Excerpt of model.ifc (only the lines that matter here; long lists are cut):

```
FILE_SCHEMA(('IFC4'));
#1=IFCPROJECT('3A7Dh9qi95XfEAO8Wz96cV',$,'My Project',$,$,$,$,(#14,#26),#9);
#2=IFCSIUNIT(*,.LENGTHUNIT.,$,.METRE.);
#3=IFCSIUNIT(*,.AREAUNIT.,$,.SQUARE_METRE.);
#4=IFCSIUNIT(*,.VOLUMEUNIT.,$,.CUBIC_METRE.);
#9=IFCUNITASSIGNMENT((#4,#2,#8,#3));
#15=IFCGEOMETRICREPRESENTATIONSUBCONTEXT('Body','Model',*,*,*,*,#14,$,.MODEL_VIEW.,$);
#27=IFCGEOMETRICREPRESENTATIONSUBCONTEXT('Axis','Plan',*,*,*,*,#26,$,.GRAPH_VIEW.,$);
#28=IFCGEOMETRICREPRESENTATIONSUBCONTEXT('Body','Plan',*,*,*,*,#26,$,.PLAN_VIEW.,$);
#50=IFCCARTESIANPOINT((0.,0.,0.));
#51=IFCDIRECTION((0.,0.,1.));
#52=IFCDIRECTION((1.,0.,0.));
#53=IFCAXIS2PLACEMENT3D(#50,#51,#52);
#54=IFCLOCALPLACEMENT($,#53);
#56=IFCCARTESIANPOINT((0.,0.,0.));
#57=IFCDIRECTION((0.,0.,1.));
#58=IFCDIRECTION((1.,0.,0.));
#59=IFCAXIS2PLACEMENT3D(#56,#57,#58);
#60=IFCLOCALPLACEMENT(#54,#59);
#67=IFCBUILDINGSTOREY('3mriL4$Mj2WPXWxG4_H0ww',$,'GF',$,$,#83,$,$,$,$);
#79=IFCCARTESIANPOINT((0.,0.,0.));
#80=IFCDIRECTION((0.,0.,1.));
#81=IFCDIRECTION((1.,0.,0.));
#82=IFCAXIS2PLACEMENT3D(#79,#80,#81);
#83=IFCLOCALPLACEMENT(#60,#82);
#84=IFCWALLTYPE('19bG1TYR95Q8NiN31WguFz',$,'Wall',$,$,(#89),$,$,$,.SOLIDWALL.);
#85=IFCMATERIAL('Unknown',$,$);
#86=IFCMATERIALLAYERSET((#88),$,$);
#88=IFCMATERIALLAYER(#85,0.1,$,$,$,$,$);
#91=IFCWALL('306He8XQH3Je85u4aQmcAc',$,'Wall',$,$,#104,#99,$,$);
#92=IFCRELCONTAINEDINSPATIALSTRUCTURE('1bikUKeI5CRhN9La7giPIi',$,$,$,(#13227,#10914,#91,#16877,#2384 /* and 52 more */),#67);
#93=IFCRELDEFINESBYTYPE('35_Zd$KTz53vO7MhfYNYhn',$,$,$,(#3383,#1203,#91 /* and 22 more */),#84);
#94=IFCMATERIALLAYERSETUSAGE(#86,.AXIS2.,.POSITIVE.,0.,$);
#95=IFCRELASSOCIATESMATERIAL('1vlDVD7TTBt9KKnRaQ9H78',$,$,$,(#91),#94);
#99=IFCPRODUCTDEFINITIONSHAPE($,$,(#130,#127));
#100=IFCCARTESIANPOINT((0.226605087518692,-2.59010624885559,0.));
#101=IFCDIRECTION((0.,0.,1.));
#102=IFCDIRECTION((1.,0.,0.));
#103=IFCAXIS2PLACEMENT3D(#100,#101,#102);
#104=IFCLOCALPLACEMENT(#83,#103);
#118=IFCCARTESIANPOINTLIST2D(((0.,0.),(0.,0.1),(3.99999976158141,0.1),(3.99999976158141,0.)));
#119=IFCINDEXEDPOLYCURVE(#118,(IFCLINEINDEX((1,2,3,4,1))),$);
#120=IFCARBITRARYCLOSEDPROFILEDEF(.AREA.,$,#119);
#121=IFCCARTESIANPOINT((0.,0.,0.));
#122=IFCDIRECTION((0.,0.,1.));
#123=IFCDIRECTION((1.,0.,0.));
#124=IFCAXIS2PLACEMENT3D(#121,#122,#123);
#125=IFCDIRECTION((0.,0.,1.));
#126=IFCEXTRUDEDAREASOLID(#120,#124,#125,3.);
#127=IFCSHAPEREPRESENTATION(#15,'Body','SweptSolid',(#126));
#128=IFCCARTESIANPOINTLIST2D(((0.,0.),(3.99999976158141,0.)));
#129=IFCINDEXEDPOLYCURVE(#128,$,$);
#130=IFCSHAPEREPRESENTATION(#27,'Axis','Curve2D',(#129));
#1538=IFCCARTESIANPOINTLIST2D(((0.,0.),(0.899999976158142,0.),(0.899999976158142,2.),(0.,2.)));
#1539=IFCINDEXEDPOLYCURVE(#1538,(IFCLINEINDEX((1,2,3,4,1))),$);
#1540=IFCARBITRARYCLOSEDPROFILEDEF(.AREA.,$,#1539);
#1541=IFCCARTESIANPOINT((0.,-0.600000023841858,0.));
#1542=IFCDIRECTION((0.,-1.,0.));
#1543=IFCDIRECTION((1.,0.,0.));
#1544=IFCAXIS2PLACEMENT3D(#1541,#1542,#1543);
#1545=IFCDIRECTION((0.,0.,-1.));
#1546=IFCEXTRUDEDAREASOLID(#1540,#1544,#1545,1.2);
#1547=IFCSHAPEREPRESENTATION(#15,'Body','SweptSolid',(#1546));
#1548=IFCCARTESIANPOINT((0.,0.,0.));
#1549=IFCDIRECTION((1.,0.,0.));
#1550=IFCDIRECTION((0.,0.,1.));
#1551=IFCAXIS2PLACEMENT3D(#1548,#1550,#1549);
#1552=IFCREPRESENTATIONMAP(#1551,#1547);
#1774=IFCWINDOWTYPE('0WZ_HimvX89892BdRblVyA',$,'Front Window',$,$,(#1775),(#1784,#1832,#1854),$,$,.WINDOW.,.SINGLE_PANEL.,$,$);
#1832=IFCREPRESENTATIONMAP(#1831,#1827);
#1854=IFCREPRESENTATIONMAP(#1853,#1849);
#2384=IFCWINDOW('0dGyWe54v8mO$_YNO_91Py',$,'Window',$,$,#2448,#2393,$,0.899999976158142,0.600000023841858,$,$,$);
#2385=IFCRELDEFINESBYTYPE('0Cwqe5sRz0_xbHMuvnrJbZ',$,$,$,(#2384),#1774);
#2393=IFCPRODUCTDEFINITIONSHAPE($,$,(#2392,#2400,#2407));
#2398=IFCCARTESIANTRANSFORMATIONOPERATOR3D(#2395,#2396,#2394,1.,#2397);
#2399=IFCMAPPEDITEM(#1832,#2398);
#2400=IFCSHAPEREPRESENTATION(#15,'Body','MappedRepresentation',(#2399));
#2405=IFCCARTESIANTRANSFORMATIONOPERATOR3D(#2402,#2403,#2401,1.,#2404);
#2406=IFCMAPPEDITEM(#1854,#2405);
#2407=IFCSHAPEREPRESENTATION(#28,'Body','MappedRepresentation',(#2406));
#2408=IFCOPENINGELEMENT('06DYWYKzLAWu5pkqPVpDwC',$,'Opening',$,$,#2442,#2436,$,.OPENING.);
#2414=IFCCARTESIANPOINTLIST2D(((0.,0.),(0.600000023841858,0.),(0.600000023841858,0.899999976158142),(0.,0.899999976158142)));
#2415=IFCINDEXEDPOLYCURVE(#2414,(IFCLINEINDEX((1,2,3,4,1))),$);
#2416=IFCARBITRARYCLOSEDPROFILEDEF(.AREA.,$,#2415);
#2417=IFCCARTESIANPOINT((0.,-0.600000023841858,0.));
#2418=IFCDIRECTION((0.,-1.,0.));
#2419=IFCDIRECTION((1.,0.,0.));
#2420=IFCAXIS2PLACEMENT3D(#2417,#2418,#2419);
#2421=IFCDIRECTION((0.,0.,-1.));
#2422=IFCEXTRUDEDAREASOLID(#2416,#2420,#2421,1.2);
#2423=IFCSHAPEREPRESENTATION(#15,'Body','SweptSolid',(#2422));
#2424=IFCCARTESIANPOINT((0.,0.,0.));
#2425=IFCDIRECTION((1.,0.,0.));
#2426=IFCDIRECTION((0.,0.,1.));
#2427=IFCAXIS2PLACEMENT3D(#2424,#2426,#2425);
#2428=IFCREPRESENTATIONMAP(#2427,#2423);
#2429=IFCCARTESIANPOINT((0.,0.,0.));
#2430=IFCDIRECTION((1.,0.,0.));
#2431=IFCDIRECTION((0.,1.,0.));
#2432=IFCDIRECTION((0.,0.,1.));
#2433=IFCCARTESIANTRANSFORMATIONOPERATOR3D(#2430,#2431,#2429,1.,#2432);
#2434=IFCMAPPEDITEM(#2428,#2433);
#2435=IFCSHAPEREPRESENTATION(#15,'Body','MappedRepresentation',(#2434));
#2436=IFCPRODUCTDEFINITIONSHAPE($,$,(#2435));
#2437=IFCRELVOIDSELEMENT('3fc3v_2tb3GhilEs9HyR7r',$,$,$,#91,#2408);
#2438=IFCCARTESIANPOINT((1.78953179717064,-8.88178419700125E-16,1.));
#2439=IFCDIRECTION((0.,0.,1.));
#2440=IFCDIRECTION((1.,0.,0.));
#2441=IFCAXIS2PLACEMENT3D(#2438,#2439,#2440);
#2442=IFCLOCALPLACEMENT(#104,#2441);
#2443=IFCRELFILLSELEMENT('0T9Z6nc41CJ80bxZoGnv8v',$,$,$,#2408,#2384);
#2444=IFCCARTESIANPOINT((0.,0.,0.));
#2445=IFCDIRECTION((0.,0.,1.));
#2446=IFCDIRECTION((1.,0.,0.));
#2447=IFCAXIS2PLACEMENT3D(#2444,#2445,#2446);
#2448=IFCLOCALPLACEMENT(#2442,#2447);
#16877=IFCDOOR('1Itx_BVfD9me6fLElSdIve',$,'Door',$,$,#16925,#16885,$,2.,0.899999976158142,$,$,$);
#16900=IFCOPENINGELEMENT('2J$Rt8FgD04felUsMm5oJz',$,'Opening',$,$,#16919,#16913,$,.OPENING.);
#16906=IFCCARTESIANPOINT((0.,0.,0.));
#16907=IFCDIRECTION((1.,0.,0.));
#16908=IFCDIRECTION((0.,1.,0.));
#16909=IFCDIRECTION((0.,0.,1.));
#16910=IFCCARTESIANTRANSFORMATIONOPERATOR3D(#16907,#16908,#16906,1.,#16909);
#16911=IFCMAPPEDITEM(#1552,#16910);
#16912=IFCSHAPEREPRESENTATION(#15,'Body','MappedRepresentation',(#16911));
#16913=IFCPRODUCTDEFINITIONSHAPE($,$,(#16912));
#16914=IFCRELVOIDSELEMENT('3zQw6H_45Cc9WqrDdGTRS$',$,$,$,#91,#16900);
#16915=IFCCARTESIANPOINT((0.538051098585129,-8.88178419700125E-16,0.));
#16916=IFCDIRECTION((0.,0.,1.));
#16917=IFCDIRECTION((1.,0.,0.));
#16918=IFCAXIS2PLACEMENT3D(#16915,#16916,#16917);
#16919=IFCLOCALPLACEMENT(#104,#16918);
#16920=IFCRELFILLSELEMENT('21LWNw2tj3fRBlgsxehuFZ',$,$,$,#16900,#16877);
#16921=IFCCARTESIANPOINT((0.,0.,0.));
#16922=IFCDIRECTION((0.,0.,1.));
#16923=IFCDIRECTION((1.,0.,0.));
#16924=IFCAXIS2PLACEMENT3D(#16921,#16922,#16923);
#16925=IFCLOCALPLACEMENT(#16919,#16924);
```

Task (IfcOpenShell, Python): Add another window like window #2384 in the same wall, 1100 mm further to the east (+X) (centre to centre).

```python
import ifcopenshell
import ifcopenshell.api.feature
import ifcopenshell.api.geometry
import ifcopenshell.api.root
import ifcopenshell.geom
import ifcopenshell.util.element
import ifcopenshell.util.placement
import ifcopenshell.util.shape
import ifcopenshell.util.unit

model = ifcopenshell.open("model.ifc")
unit_scale = ifcopenshell.util.unit.calculate_unit_scale(model)
settings = ifcopenshell.geom.settings()


def volume(element):
    """Net volume in cubic metres, openings subtracted."""
    shape = ifcopenshell.geom.create_shape(settings, element)
    return ifcopenshell.util.shape.get_volume(shape.geometry)


window = model.by_id(2384)
opening = window.FillsVoids[0].RelatingOpeningElement
wall = opening.VoidsElements[0].RelatingBuildingElement
before = volume(wall)
shift = ifcopenshell.util.placement.get_local_placement(wall.ObjectPlacement)[:3, 0] * 1.1 / unit_scale

# copy_class copies the void relationship, type, container and properties, but no geometry.
new_opening = ifcopenshell.api.root.copy_class(model, product=opening)
new_opening.Representation = ifcopenshell.util.element.copy_deep(
    model, opening.Representation, exclude=["IfcGeometricRepresentationContext", "IfcRepresentationMap"]
)
new_window = ifcopenshell.api.root.copy_class(model, product=window)
new_window.Representation = ifcopenshell.util.element.copy_deep(
    model, window.Representation, exclude=["IfcGeometricRepresentationContext", "IfcRepresentationMap"]
)
ifcopenshell.api.feature.add_filling(model, opening=new_opening, element=new_window)

for old, new in ((opening, new_opening), (window, new_window)):
    matrix = ifcopenshell.util.placement.get_local_placement(old.ObjectPlacement)
    matrix[:3, 3] += shift
    ifcopenshell.api.geometry.edit_object_placement(model, product=new, matrix=matrix, is_si=False)

after = volume(wall)

print(f"wall volume {before:.3f} -> {after:.3f} m3")

model.write("model_updated.ifc")
```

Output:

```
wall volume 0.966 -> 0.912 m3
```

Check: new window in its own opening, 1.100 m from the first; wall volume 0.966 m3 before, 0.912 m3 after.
